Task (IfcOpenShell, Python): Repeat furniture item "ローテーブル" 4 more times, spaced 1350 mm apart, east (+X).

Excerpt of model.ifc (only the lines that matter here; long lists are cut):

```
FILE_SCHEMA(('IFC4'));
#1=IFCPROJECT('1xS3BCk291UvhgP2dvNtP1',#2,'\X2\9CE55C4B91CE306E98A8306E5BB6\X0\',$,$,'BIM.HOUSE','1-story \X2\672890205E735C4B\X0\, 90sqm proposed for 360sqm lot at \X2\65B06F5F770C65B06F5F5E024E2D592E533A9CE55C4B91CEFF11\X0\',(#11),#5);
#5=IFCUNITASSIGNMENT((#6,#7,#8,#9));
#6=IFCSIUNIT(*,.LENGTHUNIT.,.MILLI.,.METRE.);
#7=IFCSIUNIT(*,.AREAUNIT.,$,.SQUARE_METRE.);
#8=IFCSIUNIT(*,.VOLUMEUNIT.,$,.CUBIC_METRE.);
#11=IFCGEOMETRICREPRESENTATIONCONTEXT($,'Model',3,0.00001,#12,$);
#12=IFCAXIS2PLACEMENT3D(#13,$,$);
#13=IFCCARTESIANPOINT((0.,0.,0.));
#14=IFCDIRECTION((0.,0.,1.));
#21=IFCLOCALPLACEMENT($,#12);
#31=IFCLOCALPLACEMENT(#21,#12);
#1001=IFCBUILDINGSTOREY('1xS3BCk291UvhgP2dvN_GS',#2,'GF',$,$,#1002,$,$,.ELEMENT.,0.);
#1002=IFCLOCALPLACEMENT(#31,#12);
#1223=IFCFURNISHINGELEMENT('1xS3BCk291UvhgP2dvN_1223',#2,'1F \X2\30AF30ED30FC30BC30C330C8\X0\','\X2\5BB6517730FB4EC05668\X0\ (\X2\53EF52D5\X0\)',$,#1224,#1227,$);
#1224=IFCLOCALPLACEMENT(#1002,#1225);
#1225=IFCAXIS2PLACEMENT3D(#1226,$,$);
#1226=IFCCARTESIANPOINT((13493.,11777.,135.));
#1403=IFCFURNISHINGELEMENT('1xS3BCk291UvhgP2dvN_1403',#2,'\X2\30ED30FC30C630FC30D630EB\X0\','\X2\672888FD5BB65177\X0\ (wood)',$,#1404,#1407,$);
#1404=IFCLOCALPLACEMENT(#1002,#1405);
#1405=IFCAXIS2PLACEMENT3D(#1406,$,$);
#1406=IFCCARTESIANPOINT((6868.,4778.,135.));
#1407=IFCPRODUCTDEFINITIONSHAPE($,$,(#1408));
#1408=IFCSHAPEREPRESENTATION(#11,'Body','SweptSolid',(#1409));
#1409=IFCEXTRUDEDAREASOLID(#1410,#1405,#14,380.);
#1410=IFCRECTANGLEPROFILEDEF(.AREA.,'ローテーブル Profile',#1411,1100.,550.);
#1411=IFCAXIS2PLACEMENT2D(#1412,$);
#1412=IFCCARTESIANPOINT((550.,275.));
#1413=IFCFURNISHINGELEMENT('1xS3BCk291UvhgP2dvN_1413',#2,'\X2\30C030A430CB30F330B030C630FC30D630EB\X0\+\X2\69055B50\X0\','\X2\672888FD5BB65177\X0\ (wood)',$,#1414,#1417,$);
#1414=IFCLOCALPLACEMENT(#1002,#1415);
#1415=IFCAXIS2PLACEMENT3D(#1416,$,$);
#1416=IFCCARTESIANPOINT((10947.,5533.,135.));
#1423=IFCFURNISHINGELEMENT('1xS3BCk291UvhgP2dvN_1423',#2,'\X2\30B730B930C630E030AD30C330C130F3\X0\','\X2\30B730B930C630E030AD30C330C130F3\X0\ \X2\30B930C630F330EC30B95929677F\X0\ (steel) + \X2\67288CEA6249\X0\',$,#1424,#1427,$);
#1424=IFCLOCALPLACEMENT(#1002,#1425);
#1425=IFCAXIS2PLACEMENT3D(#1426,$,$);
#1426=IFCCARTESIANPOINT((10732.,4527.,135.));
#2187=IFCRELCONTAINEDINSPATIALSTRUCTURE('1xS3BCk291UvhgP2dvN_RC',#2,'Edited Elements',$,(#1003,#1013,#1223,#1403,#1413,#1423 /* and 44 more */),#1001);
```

```python
import numpy as np
import ifcopenshell
import ifcopenshell.api.geometry
import ifcopenshell.api.root
import ifcopenshell.util.element
import ifcopenshell.util.placement
import ifcopenshell.util.unit

model = ifcopenshell.open("model.ifc")
unit_scale = ifcopenshell.util.unit.calculate_unit_scale(model)


def reuse_history(source, copy):
    """copy_class also copies each property set's owner history, people and application; keep the originals."""
    for rel in copy.IsDefinedBy:
        if rel.is_a("IfcRelDefinesByProperties") and (history := rel.RelatingPropertyDefinition.OwnerHistory):
            rel.RelatingPropertyDefinition.OwnerHistory = source.OwnerHistory
            ifcopenshell.util.element.remove_deep2(model, history)


source = model.by_id(1403)
base = ifcopenshell.util.placement.get_local_placement(source.ObjectPlacement)
step = np.array([1.0, 0.0, 0.0]) * 1.35 / unit_scale

for i in range(1, 5):
    copy = ifcopenshell.api.root.copy_class(model, product=source)
    copy.Representation = ifcopenshell.util.element.copy_deep(
        model, source.Representation, exclude=["IfcGeometricRepresentationContext", "IfcRepresentationMap"]
    )
    reuse_history(source, copy)
    matrix = base.copy()
    matrix[:3, 3] += i * step
    print("added at", matrix[:3, 3].round(3) + 0.0)
    ifcopenshell.api.geometry.edit_object_placement(model, product=copy, matrix=matrix, is_si=False)

model.write("model_v2.ifc")
```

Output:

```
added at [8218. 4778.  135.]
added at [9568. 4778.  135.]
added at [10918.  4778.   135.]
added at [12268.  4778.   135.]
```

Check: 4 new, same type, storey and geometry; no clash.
